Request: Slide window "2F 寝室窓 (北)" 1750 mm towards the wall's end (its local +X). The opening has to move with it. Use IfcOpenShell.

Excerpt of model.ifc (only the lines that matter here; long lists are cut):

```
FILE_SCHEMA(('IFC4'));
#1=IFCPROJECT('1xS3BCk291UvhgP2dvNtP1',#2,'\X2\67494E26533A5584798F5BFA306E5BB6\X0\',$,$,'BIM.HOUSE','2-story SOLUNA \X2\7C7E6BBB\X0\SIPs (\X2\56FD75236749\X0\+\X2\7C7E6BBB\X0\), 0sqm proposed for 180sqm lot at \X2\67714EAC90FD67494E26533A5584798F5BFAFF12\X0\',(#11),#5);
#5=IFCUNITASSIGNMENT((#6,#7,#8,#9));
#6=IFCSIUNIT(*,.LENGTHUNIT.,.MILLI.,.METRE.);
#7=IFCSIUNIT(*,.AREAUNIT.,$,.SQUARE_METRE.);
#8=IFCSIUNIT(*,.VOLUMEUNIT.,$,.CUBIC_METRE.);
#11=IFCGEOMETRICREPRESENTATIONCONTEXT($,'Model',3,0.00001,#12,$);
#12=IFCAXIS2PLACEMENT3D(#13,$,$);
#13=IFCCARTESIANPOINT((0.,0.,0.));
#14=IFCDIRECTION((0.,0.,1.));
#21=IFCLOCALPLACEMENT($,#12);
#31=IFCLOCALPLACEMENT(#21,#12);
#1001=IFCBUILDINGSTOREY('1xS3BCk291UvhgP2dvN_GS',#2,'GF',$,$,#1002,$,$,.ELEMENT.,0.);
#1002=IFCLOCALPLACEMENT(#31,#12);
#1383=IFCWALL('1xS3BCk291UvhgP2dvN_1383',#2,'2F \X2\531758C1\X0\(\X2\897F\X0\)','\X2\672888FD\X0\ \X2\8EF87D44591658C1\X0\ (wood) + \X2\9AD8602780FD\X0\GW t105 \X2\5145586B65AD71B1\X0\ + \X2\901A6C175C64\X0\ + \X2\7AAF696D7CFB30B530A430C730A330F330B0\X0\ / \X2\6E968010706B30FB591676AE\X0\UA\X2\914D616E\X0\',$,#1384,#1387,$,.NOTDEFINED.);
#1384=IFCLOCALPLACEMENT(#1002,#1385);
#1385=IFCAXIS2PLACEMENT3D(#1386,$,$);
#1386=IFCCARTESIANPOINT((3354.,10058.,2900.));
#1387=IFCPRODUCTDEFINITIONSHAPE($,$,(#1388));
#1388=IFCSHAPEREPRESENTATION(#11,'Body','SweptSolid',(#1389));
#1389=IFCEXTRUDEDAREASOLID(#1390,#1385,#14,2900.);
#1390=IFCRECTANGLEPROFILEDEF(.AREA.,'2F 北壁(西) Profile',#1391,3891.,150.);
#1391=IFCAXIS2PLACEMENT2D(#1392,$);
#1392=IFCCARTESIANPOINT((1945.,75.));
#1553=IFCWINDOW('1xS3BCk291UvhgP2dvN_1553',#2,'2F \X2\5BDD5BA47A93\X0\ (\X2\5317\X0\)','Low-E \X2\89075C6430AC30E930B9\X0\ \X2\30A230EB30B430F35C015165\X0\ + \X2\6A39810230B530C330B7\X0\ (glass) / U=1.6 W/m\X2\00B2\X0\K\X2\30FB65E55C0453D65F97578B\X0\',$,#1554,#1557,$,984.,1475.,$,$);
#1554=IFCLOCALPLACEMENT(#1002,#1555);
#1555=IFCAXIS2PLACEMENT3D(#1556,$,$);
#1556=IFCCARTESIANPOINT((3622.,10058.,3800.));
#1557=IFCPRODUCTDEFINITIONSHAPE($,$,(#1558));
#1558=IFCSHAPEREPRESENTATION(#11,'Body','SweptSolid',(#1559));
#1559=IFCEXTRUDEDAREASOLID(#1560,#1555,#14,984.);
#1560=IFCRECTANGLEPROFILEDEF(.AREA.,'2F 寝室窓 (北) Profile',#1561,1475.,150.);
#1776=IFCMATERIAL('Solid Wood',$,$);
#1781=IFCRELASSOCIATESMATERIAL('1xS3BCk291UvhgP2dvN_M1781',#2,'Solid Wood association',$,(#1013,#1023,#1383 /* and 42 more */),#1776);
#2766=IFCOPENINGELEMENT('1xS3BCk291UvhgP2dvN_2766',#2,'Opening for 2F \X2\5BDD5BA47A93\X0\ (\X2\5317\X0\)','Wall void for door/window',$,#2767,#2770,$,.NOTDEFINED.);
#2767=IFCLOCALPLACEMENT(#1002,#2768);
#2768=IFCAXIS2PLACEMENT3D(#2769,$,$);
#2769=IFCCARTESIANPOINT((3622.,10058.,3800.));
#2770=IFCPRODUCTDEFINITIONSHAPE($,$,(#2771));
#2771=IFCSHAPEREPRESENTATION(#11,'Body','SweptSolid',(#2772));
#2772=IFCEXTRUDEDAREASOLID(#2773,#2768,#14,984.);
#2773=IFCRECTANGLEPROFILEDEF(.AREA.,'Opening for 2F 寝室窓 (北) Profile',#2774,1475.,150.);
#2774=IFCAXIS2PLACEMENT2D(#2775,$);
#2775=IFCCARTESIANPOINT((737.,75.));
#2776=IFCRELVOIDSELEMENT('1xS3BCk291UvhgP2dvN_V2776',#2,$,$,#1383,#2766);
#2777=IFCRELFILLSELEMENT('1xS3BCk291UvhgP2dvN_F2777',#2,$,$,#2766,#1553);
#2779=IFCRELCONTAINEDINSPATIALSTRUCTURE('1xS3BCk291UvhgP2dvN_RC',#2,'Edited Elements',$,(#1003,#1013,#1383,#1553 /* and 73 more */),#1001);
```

```python
import ifcopenshell
import ifcopenshell.api.geometry
import ifcopenshell.util.placement
import ifcopenshell.util.unit

model = ifcopenshell.open("model.ifc")
unit_scale = ifcopenshell.util.unit.calculate_unit_scale(model)

window = model.by_guid("1xS3BCk291UvhgP2dvN_1553")
opening = window.FillsVoids[0].RelatingOpeningElement
wall = opening.VoidsElements[0].RelatingBuildingElement

wall_matrix = ifcopenshell.util.placement.get_local_placement(wall.ObjectPlacement)
shift = wall_matrix[:3, 0] * 1.75 / unit_scale
before = ifcopenshell.util.placement.get_local_placement(window.ObjectPlacement)[:3, 3].copy()

# The window is not placed relative to its opening, so move both.
for product in (opening, window):
    matrix = ifcopenshell.util.placement.get_local_placement(product.ObjectPlacement)
    matrix[:3, 3] += shift
    ifcopenshell.api.geometry.edit_object_placement(model, product=product, matrix=matrix, is_si=False)

after = ifcopenshell.util.placement.get_local_placement(window.ObjectPlacement)[:3, 3]
print("window moved by", (after - before).round(3) + 0.0)

model.write("model-out.ifc")
```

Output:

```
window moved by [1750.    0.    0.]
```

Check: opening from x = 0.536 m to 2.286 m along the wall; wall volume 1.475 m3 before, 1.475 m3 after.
